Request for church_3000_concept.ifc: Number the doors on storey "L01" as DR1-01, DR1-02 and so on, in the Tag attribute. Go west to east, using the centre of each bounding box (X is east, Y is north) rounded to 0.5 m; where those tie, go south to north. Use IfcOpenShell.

First a look at what the model holds.

```python
import ifcopenshell
import ifcopenshell.util.element
import ifcopenshell.util.placement

model = ifcopenshell.open("church_3000_concept.ifc")
print(model.schema)
storey = next(s for s in model.by_type("IfcBuildingStorey") if s.Name == "L01")
doors = [e for e in ifcopenshell.util.element.get_decomposition(storey) if e.is_a("IfcDoor")]
for e in sorted(doors, key=lambda e: e.id()):
    origin = ifcopenshell.util.placement.get_local_placement(e.ObjectPlacement)[:3, 3]
    print(e.id(), e.Tag, e.Name, origin.round(2) + 0.0, sep=" | ")
```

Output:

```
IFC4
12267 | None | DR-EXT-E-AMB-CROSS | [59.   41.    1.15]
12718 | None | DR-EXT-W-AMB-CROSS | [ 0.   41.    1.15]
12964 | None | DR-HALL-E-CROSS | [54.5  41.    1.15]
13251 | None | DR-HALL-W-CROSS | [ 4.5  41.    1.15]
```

```python
import ifcopenshell
import ifcopenshell.geom
import ifcopenshell.util.element
import ifcopenshell.util.shape

model = ifcopenshell.open("church_3000_concept.ifc")
settings = ifcopenshell.geom.settings()
settings.set("use-world-coords", True)


def centre(element):
    shape = ifcopenshell.geom.create_shape(settings, element)
    return ifcopenshell.util.shape.get_bbox_centroid(shape.geometry)


storey = next(s for s in model.by_type("IfcBuildingStorey") if s.Name == "L01")
doors = [e for e in ifcopenshell.util.element.get_decomposition(storey) if e.is_a("IfcDoor")]

# Insertion points can sit at a corner or the storey origin, so sort by the geometry (in metres).
centres = {e: centre(e) for e in doors}
doors.sort(key=lambda e: (round(centres[e][0] / 0.5), centres[e][1]))

for i, e in enumerate(doors, start=1):
    number = f"DR1-{i:02d}"
    e.Tag = number
    print(e.id(), number)

model.write("church_3000_concept_v2.ifc")
```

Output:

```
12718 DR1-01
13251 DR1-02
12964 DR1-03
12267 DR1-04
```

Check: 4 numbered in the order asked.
